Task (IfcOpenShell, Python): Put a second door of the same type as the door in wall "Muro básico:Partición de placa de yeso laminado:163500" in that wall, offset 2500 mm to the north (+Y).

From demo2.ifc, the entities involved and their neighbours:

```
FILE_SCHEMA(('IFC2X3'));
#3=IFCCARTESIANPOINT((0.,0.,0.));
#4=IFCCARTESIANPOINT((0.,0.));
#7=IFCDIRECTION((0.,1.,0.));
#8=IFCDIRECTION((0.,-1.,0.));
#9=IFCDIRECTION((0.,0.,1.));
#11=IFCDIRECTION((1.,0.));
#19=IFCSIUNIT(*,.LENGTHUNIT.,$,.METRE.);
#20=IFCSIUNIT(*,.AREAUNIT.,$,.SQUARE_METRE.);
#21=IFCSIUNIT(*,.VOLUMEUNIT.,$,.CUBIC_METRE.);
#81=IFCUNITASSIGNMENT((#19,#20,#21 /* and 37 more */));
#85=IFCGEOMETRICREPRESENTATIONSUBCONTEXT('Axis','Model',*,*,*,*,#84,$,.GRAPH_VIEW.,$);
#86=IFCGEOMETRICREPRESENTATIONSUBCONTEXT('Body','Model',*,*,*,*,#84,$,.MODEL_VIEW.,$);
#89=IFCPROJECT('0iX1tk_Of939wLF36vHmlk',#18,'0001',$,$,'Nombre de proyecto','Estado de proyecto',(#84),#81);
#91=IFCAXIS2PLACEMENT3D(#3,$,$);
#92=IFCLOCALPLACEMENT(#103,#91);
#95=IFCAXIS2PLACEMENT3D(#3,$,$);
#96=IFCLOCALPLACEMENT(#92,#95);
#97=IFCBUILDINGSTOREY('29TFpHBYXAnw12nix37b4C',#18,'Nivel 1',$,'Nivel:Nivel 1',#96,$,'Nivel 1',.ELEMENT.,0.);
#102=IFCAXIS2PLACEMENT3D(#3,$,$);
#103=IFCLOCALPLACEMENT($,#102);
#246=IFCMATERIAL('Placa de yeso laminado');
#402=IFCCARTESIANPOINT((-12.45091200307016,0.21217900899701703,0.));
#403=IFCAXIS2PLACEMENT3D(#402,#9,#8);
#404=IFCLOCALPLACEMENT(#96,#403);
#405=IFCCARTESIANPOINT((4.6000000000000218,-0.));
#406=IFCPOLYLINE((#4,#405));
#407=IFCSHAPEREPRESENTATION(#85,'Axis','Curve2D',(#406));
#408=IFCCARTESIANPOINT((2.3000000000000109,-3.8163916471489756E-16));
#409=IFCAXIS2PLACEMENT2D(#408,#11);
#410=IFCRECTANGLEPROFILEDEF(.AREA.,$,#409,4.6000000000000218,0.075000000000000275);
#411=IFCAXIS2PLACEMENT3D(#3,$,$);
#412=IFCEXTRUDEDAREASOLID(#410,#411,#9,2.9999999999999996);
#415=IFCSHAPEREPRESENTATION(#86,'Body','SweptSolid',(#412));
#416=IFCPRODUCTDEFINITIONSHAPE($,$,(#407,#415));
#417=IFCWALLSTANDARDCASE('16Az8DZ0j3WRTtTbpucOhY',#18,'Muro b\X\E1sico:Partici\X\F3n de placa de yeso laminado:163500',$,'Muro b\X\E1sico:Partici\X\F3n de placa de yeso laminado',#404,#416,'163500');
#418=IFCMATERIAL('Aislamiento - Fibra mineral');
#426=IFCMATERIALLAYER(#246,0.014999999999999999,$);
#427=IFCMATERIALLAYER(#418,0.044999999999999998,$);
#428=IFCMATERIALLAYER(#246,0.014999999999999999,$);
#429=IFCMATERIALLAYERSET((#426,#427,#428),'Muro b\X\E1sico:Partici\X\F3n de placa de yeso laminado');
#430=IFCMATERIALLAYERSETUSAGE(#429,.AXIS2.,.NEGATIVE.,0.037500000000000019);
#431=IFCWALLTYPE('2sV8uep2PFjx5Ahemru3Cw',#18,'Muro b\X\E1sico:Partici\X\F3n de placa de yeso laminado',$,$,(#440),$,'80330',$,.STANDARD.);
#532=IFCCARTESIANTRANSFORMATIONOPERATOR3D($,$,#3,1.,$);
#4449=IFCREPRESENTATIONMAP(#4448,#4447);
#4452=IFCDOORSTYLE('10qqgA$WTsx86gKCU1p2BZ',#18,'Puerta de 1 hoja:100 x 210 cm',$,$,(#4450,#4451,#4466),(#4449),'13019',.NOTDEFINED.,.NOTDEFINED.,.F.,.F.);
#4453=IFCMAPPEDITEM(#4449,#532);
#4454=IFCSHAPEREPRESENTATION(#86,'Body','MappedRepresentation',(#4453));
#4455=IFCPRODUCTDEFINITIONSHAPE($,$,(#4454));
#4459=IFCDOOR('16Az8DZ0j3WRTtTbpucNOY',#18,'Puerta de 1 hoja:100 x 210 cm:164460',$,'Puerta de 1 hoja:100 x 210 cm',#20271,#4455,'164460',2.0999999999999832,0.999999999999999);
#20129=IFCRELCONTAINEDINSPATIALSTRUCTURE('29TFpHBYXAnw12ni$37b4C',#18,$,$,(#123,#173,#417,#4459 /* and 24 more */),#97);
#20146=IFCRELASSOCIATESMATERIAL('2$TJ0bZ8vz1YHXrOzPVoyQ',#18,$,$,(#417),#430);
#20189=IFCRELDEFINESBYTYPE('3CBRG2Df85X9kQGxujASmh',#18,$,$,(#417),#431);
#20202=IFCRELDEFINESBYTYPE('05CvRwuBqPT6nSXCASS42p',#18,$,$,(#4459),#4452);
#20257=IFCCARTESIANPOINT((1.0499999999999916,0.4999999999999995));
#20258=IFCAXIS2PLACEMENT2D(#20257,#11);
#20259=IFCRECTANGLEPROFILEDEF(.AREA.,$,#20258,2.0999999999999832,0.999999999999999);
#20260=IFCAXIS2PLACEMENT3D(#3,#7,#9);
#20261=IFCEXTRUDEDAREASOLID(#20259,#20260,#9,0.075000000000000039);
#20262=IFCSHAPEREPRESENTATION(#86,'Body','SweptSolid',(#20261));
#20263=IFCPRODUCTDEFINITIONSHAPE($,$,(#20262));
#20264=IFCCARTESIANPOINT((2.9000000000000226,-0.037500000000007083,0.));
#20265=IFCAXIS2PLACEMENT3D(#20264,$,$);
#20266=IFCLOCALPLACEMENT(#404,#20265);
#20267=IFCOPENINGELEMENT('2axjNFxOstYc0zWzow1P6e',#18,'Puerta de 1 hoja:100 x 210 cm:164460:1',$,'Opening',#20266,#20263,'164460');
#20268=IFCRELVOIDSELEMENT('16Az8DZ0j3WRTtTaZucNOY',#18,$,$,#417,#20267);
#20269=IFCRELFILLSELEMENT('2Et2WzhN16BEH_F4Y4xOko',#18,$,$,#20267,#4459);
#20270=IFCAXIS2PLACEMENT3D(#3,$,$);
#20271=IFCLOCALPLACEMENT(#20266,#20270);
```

```python
import ifcopenshell
import ifcopenshell.api.feature
import ifcopenshell.api.geometry
import ifcopenshell.api.root
import ifcopenshell.geom
import ifcopenshell.util.element
import ifcopenshell.util.placement
import ifcopenshell.util.shape
import ifcopenshell.util.unit

model = ifcopenshell.open("demo2.ifc")
unit_scale = ifcopenshell.util.unit.calculate_unit_scale(model)
settings = ifcopenshell.geom.settings()


def volume(element):
    """Net volume in cubic metres, openings subtracted."""
    shape = ifcopenshell.geom.create_shape(settings, element)
    return ifcopenshell.util.shape.get_volume(shape.geometry)


def reuse_history(source, copy):
    """copy_class also copies each property set's owner history, people and application; keep the originals."""
    for rel in copy.IsDefinedBy:
        if rel.is_a("IfcRelDefinesByProperties") and (history := rel.RelatingPropertyDefinition.OwnerHistory):
            rel.RelatingPropertyDefinition.OwnerHistory = source.OwnerHistory
            ifcopenshell.util.element.remove_deep2(model, history)


door = model.by_id(4459)
opening = door.FillsVoids[0].RelatingOpeningElement
wall = opening.VoidsElements[0].RelatingBuildingElement
before = volume(wall)
shift = ifcopenshell.util.placement.get_local_placement(wall.ObjectPlacement)[:3, 0] * -2.5 / unit_scale

# copy_class copies the void relationship, type, container and properties, but no geometry.
new_opening = ifcopenshell.api.root.copy_class(model, product=opening)
new_opening.Representation = ifcopenshell.util.element.copy_deep(
    model, opening.Representation, exclude=["IfcGeometricRepresentationContext", "IfcRepresentationMap"]
)
new_opening.Name = "Puerta de 1 hoja:100 x 210 cm"
new_opening.Tag = None
new_door = ifcopenshell.api.root.copy_class(model, product=door)
new_door.Representation = ifcopenshell.util.element.copy_deep(
    model, door.Representation, exclude=["IfcGeometricRepresentationContext", "IfcRepresentationMap"]
)
new_door.Name = "Puerta de 1 hoja:100 x 210 cm"
new_door.Tag = None
reuse_history(door, new_door)
fills = ifcopenshell.api.feature.add_filling(model, opening=new_opening, element=new_door)
fills.OwnerHistory = new_door.OwnerHistory  # required in IFC2X3

for old, new in ((opening, new_opening), (door, new_door)):
    matrix = ifcopenshell.util.placement.get_local_placement(old.ObjectPlacement)
    matrix[:3, 3] += shift
    ifcopenshell.api.geometry.edit_object_placement(model, product=new, matrix=matrix, is_si=False)

after = volume(wall)

print(f"wall volume {before:.3f} -> {after:.3f} m3")

model.write("demo2_v2.ifc")
```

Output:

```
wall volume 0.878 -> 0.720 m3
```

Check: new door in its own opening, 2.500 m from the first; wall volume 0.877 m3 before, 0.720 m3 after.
